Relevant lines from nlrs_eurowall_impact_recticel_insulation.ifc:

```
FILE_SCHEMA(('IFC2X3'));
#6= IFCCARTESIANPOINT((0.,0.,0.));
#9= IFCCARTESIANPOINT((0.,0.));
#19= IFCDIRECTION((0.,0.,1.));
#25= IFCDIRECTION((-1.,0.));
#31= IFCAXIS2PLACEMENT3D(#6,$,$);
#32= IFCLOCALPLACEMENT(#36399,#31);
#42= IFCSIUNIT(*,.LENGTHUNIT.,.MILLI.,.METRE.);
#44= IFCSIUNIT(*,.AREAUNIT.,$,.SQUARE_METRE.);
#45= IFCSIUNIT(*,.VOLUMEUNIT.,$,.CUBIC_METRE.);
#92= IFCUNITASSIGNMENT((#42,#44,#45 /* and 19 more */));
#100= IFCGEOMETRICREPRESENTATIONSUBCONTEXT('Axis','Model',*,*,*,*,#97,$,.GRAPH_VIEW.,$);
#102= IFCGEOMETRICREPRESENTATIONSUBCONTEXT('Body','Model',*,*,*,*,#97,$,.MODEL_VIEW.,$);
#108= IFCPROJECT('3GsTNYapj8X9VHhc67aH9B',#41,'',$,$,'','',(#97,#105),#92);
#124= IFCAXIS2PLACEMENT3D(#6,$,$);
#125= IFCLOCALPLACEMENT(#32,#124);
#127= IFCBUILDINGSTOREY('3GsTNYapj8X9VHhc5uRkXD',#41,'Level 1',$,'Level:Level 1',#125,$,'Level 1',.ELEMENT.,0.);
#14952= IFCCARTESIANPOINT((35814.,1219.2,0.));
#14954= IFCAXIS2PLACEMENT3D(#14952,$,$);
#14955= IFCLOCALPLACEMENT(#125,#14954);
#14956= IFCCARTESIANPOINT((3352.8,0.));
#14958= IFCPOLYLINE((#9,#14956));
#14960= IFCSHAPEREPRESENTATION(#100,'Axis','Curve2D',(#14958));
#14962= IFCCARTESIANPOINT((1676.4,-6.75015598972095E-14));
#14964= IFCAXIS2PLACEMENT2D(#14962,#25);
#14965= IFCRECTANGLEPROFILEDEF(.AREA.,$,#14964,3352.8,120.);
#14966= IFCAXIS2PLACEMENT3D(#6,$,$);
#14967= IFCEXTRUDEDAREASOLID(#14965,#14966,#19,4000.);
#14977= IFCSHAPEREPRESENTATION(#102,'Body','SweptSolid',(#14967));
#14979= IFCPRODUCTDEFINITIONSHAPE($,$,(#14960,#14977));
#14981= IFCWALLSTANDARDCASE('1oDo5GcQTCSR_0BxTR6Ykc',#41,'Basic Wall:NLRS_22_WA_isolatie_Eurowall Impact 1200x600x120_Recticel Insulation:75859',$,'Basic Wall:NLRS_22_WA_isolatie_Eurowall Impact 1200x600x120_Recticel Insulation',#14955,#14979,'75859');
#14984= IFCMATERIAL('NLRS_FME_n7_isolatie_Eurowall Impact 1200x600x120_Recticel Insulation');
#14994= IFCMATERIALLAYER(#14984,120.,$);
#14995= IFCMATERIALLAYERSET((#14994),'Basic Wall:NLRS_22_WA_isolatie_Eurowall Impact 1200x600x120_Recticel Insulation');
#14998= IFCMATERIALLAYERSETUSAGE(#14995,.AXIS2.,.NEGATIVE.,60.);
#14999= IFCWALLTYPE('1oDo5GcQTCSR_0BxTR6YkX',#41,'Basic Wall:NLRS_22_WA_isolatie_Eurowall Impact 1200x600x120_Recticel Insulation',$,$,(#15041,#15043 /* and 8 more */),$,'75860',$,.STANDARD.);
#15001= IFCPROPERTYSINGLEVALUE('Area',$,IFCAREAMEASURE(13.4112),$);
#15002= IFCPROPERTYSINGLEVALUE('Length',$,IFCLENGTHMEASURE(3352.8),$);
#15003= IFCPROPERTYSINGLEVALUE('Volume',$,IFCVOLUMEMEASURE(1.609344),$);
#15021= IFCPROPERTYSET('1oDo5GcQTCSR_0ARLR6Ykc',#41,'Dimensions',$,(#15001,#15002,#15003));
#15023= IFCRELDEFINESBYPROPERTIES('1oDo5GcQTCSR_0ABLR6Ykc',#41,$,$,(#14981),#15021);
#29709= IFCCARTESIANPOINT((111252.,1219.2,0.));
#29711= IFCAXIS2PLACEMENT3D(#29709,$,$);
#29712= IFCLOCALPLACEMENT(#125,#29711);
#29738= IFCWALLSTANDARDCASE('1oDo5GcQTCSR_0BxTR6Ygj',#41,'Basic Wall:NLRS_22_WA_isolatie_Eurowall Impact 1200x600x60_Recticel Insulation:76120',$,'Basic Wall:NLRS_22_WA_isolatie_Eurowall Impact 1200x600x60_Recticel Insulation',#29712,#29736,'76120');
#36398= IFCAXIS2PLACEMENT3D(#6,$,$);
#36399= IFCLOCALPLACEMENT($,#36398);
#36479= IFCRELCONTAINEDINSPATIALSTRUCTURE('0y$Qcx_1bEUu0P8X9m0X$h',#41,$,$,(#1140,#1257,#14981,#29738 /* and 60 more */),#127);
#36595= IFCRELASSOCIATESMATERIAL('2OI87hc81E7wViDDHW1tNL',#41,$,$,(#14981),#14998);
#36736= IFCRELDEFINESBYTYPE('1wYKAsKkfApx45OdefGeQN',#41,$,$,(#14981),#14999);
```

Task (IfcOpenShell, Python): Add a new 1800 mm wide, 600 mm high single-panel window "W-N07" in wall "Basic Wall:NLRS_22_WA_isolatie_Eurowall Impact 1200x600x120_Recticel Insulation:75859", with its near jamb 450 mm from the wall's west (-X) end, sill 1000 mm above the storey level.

```python
import numpy as np
import ifcopenshell
import ifcopenshell.api.feature
import ifcopenshell.api.geometry
import ifcopenshell.api.pset
import ifcopenshell.api.root
import ifcopenshell.api.spatial
import ifcopenshell.api.type
import ifcopenshell.geom
import ifcopenshell.util.element
import ifcopenshell.util.placement
import ifcopenshell.util.representation
import ifcopenshell.util.shape
import ifcopenshell.util.unit

model = ifcopenshell.open("nlrs_eurowall_impact_recticel_insulation.ifc")
unit_scale = ifcopenshell.util.unit.calculate_unit_scale(model)
area_scale = ifcopenshell.util.unit.calculate_unit_scale(model, "AREAUNIT")
volume_scale = ifcopenshell.util.unit.calculate_unit_scale(model, "VOLUMEUNIT")
settings = ifcopenshell.geom.settings()


def volume(element):
    """Net volume in cubic metres, openings subtracted."""
    shape = ifcopenshell.geom.create_shape(settings, element)
    return ifcopenshell.util.shape.get_volume(shape.geometry)


wall = model.by_guid("1oDo5GcQTCSR_0BxTR6Ykc")
storey = ifcopenshell.util.element.get_container(wall, ifc_class="IfcBuildingStorey")
context = ifcopenshell.util.representation.get_context(model, "Model", "Body", "MODEL_VIEW")
before = volume(wall)

width, height, from_end, sill = 1.8, 0.6, 0.45, 1  # metres

# The wall runs along its own X axis, and the end named is its -X end.
wall_shape = ifcopenshell.geom.create_shape(settings, wall)
x, y, z = ifcopenshell.util.shape.get_vertices(wall_shape.geometry).T
start = x.min() + from_end
face, thickness = float(y.min()), float(y.max() - y.min())
wall_matrix = ifcopenshell.util.placement.get_local_placement(wall.ObjectPlacement)
level = ifcopenshell.util.placement.get_local_placement(storey.ObjectPlacement)[2, 3]


def in_wall(x, y):
    """Placement at x, y metres in the wall's axes, at sill height."""
    matrix = wall_matrix.copy()
    matrix[:, 3] = wall_matrix @ np.array([x / unit_scale, y / unit_scale, 0.0, 1.0])
    matrix[2, 3] = level + sill / unit_scale
    return matrix


# Opening: a box that overshoots both wall faces by 50 mm.
opening = ifcopenshell.api.root.create_entity(model, ifc_class="IfcOpeningElement")
box = ifcopenshell.api.geometry.add_wall_representation(
    model, context=context, length=width, height=height, thickness=thickness + 0.1
)
ifcopenshell.api.geometry.assign_representation(model, product=opening, representation=box)
ifcopenshell.api.geometry.edit_object_placement(model, product=opening, matrix=in_wall(start, face - 0.05), is_si=False)
ifcopenshell.api.feature.add_feature(model, feature=opening, element=wall)

window = ifcopenshell.api.root.create_entity(model, ifc_class="IfcWindow", name="W-N07")
window.OverallWidth, window.OverallHeight = width / unit_scale, height / unit_scale
body = ifcopenshell.api.geometry.add_window_representation(
    model,
    context=context,
    overall_width=window.OverallWidth,
    overall_height=window.OverallHeight,
    partition_type="SINGLE_PANEL",
)
ifcopenshell.api.geometry.assign_representation(model, product=window, representation=body)
ifcopenshell.api.spatial.assign_container(model, products=[window], relating_structure=storey)
fills = ifcopenshell.api.feature.add_filling(model, opening=opening, element=window)
fills.OwnerHistory = window.OwnerHistory  # required in IFC2X3

# IFC2X3 keeps the operation on the window style.
style = ifcopenshell.api.root.create_entity(model, ifc_class="IfcWindowStyle", name="W-N07")
style.OperationType, style.ConstructionType = "SINGLE_PANEL", "NOTDEFINED"
style.ParameterTakesPrecedence = style.Sizeable = False
ifcopenshell.api.type.assign_type(model, related_objects=[window], relating_type=style)

# Centre the window in the wall's thickness.
ifcopenshell.api.geometry.edit_object_placement(model, product=window, matrix=in_wall(start, face), is_si=False)
window_shape = ifcopenshell.geom.create_shape(settings, window)
depth = ifcopenshell.util.shape.get_vertices(window_shape.geometry)[:, 1]
offset = face + thickness / 2 - (depth.min() + depth.max()) / 2
ifcopenshell.api.geometry.edit_object_placement(model, product=window, matrix=in_wall(start, offset), is_si=False)

after = volume(wall)

# Update the wall's stored quantities.
pset = model.by_id(ifcopenshell.util.element.get_pset(wall, "Dimensions", should_inherit=False)["id"])
ifcopenshell.api.pset.edit_pset(model, pset=pset, properties={
    "Area": model.create_entity("IfcAreaMeasure", after / thickness / area_scale),
    "Volume": model.create_entity("IfcVolumeMeasure", after / volume_scale),
})

print(f"wall volume {before:.3f} -> {after:.3f} m3")

model.write("nlrs_eurowall_impact_recticel_insulation_rev.ifc")
```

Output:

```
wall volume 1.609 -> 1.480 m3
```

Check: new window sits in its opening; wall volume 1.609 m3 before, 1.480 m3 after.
